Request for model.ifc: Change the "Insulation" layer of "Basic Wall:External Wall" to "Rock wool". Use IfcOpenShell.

First a look at what the model holds.

```python
import ifcopenshell
import ifcopenshell.util.element

model = ifcopenshell.open("model.ifc")
print(model.schema)
for layer_set in model.by_type("IfcMaterialLayerSet"):
    if layer_set.LayerSetName == "Basic Wall:External Wall":
        for layer in layer_set.MaterialLayers:
            print(layer.id(), layer.Material and layer.Material.Name, layer.LayerThickness, sep=" | ")
        print(len(ifcopenshell.util.element.get_elements_by_material(model, layer_set)), "elements and types use it")
print(sorted(m.Name for m in model.by_type("IfcMaterial") if m.Name)[:60])
```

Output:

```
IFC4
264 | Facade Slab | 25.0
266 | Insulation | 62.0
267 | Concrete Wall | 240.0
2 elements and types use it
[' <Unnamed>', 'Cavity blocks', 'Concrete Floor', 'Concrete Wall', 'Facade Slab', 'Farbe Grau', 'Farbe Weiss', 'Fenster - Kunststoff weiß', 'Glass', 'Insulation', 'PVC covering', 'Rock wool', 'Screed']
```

```python
import ifcopenshell
import ifcopenshell.api.material

model = ifcopenshell.open("model.ifc")

layer_set = next(s for s in model.by_type("IfcMaterialLayerSet") if s.LayerSetName == "Basic Wall:External Wall")
layer = next(l for l in layer_set.MaterialLayers if l.Material and l.Material.Name == "Insulation")
material = next(m for m in model.by_type("IfcMaterial") if m.Name == "Rock wool")

# Point this one layer at the other material; renaming the old one would change it everywhere.
ifcopenshell.api.material.edit_layer(model, layer=layer, attributes={}, material=material)

print([l.Material.Name if l.Material else None for l in layer_set.MaterialLayers])

model.write("model_edited.ifc")
```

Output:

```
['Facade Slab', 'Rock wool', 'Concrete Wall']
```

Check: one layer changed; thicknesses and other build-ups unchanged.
